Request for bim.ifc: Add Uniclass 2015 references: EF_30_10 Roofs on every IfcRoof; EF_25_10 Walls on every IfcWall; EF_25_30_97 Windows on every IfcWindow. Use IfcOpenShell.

First a look at what the model holds.

```python
import ifcopenshell

model = ifcopenshell.open("bim.ifc")
print(model.schema)
print("classifications:", [c.Name for c in model.by_type("IfcClassification")])
for ifc_class in ("IfcDoor", "IfcRoof", "IfcStair", "IfcWall", "IfcWindow"):
    print(ifc_class, len(model.by_type(ifc_class)))
```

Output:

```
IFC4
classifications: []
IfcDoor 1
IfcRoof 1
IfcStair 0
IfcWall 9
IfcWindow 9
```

```python
import ifcopenshell
import ifcopenshell.api.classification

model = ifcopenshell.open("bim.ifc")

system = ifcopenshell.api.classification.add_classification(model, classification="Uniclass 2015")

codes = {
    "IfcRoof": ("EF_30_10", "Roofs"),
    "IfcWall": ("EF_25_10", "Walls"),
    "IfcWindow": ("EF_25_30_97", "Windows"),
}
for ifc_class, (code, name) in codes.items():
    products = model.by_type(ifc_class)
    ifcopenshell.api.classification.add_reference(
        model, products=products, classification=system, identification=code, name=name
    )
    print(code, len(products))

model.write("bim_updated.ifc")
```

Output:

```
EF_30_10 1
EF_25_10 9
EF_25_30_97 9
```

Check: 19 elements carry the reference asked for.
